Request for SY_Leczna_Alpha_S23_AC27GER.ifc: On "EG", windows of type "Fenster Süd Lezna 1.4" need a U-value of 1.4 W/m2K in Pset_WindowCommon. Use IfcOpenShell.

First a look at what the model holds.

```python
import ifcopenshell
import ifcopenshell.util.element

model = ifcopenshell.open("SY_Leczna_Alpha_S23_AC27GER.ifc")
print(model.schema)
storey = next(s for s in model.by_type("IfcBuildingStorey") if s.Name == "EG")
windows = [e for e in ifcopenshell.util.element.get_decomposition(storey) if e.is_a("IfcWindow")]
seen = {}
for e in windows:
    element_type = ifcopenshell.util.element.get_type(e)
    key = (element_type.Name if element_type != e and element_type else None, ifcopenshell.util.element.get_pset(e, "Pset_WindowCommon", "ThermalTransmittance"))
    seen[key] = seen.get(key, 0) + 1
for (name, value), count in sorted(seen.items(), key=str):
    print(count, "x", name, "|", value)
```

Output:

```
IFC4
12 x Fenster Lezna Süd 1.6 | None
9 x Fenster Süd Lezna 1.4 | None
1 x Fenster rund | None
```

```python
import ifcopenshell
import ifcopenshell.api.pset
import ifcopenshell.util.element

model = ifcopenshell.open("SY_Leczna_Alpha_S23_AC27GER.ifc")

storey = next(s for s in model.by_type("IfcBuildingStorey") if s.Name == "EG")
windows = [e for e in ifcopenshell.util.element.get_decomposition(storey) if e.is_a("IfcWindow")]

count = 0
for e in windows:
    element_type = ifcopenshell.util.element.get_type(e)
    if element_type in (None, e) or element_type.Name != "Fenster Süd Lezna 1.4":
        continue
    # add_pset returns the element's existing set when there is one.
    pset = ifcopenshell.api.pset.add_pset(model, product=e, name="Pset_WindowCommon")
    ifcopenshell.api.pset.edit_pset(model, pset=pset, properties={"ThermalTransmittance": 1.4})
    count += 1

print(count, "windows updated")

model.write("SY_Leczna_Alpha_S23_AC27GER_rev.ifc")
```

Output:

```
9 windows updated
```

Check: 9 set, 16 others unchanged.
